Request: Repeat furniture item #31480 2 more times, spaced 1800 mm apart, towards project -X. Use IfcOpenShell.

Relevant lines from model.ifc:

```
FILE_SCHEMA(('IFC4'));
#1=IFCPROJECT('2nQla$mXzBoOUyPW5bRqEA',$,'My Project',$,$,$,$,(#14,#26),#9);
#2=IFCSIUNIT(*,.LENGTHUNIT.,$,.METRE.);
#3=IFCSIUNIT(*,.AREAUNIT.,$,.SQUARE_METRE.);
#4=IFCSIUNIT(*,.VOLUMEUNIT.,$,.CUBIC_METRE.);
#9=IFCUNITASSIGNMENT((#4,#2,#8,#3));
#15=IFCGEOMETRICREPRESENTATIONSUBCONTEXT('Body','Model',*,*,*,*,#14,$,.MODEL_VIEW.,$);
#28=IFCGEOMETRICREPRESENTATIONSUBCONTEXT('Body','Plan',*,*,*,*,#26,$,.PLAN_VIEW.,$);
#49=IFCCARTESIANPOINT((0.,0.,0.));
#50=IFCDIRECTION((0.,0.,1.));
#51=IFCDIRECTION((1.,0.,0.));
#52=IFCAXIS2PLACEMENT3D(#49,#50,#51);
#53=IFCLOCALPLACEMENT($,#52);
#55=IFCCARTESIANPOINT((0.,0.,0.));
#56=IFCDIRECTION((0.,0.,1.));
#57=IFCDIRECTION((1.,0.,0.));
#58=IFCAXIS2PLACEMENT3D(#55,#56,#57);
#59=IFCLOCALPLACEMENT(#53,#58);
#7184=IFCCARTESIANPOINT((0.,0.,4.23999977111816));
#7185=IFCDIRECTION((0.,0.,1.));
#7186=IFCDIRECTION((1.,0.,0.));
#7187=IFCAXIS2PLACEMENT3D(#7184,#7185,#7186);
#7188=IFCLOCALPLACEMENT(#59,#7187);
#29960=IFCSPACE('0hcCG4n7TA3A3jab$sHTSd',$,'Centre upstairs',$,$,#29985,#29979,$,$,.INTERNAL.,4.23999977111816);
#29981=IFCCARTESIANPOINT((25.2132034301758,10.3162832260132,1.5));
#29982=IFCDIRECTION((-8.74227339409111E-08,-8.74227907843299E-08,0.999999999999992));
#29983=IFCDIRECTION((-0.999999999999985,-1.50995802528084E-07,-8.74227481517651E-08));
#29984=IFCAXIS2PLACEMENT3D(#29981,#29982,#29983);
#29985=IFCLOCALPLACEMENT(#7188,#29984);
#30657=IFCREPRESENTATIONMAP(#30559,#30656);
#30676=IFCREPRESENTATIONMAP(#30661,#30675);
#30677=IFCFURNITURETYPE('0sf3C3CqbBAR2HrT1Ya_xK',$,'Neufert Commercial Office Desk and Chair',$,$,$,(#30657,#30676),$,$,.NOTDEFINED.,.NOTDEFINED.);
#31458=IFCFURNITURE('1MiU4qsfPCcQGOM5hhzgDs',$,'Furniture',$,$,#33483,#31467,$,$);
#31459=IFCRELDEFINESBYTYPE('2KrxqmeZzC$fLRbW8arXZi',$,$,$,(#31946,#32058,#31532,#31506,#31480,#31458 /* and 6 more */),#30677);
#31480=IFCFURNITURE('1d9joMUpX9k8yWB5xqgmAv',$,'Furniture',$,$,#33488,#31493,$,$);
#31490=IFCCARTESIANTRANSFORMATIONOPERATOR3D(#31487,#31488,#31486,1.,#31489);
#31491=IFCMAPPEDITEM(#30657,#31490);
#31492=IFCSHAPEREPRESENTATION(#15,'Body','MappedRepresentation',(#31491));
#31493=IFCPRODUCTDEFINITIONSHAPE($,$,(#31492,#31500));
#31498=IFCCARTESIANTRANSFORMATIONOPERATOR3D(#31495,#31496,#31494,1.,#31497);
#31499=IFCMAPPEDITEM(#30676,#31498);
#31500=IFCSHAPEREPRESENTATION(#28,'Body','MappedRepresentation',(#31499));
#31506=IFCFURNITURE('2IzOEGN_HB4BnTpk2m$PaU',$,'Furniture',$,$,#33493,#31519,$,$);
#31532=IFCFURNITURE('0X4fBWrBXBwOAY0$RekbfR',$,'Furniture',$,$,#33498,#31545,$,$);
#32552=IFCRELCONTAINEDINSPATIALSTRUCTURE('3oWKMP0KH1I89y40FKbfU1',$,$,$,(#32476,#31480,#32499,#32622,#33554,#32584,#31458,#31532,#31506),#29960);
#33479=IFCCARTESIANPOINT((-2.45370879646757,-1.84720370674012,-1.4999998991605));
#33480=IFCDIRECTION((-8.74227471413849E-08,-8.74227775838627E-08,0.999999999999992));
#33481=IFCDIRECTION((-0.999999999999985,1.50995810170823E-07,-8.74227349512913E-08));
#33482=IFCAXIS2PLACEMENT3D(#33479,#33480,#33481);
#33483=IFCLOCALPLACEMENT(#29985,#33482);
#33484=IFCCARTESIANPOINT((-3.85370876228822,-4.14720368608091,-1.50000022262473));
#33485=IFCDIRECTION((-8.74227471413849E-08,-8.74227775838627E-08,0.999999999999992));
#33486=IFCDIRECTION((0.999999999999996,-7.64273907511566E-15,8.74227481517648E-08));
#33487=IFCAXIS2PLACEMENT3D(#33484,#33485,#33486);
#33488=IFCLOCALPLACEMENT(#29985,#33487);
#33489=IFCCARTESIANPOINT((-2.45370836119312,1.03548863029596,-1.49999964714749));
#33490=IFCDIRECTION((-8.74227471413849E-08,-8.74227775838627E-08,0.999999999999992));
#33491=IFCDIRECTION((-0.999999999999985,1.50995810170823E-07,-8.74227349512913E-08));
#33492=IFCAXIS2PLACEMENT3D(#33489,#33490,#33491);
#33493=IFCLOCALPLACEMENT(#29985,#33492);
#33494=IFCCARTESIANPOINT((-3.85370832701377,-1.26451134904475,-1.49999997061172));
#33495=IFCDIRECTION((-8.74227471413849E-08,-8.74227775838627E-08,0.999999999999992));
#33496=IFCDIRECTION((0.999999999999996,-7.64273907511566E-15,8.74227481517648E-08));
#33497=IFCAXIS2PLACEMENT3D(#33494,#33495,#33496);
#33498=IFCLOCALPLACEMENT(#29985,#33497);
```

```python
import numpy as np
import ifcopenshell
import ifcopenshell.api.geometry
import ifcopenshell.api.root
import ifcopenshell.util.element
import ifcopenshell.util.placement
import ifcopenshell.util.unit

model = ifcopenshell.open("model.ifc")
unit_scale = ifcopenshell.util.unit.calculate_unit_scale(model)

source = model.by_guid("1d9joMUpX9k8yWB5xqgmAv")
base = ifcopenshell.util.placement.get_local_placement(source.ObjectPlacement)
step = np.array([-1.0, 0.0, 0.0]) * 1.8 / unit_scale

for i in range(1, 3):
    copy = ifcopenshell.api.root.copy_class(model, product=source)
    copy.Representation = ifcopenshell.util.element.copy_deep(
        model, source.Representation, exclude=["IfcGeometricRepresentationContext", "IfcRepresentationMap"]
    )
    matrix = base.copy()
    matrix[:3, 3] += i * step
    print("added at", matrix[:3, 3].round(3) + 0.0)
    ifcopenshell.api.geometry.edit_object_placement(model, product=copy, matrix=matrix, is_si=False)

model.write("model_v2.ifc")
```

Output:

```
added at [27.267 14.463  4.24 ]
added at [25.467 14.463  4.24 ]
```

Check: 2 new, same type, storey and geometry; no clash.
